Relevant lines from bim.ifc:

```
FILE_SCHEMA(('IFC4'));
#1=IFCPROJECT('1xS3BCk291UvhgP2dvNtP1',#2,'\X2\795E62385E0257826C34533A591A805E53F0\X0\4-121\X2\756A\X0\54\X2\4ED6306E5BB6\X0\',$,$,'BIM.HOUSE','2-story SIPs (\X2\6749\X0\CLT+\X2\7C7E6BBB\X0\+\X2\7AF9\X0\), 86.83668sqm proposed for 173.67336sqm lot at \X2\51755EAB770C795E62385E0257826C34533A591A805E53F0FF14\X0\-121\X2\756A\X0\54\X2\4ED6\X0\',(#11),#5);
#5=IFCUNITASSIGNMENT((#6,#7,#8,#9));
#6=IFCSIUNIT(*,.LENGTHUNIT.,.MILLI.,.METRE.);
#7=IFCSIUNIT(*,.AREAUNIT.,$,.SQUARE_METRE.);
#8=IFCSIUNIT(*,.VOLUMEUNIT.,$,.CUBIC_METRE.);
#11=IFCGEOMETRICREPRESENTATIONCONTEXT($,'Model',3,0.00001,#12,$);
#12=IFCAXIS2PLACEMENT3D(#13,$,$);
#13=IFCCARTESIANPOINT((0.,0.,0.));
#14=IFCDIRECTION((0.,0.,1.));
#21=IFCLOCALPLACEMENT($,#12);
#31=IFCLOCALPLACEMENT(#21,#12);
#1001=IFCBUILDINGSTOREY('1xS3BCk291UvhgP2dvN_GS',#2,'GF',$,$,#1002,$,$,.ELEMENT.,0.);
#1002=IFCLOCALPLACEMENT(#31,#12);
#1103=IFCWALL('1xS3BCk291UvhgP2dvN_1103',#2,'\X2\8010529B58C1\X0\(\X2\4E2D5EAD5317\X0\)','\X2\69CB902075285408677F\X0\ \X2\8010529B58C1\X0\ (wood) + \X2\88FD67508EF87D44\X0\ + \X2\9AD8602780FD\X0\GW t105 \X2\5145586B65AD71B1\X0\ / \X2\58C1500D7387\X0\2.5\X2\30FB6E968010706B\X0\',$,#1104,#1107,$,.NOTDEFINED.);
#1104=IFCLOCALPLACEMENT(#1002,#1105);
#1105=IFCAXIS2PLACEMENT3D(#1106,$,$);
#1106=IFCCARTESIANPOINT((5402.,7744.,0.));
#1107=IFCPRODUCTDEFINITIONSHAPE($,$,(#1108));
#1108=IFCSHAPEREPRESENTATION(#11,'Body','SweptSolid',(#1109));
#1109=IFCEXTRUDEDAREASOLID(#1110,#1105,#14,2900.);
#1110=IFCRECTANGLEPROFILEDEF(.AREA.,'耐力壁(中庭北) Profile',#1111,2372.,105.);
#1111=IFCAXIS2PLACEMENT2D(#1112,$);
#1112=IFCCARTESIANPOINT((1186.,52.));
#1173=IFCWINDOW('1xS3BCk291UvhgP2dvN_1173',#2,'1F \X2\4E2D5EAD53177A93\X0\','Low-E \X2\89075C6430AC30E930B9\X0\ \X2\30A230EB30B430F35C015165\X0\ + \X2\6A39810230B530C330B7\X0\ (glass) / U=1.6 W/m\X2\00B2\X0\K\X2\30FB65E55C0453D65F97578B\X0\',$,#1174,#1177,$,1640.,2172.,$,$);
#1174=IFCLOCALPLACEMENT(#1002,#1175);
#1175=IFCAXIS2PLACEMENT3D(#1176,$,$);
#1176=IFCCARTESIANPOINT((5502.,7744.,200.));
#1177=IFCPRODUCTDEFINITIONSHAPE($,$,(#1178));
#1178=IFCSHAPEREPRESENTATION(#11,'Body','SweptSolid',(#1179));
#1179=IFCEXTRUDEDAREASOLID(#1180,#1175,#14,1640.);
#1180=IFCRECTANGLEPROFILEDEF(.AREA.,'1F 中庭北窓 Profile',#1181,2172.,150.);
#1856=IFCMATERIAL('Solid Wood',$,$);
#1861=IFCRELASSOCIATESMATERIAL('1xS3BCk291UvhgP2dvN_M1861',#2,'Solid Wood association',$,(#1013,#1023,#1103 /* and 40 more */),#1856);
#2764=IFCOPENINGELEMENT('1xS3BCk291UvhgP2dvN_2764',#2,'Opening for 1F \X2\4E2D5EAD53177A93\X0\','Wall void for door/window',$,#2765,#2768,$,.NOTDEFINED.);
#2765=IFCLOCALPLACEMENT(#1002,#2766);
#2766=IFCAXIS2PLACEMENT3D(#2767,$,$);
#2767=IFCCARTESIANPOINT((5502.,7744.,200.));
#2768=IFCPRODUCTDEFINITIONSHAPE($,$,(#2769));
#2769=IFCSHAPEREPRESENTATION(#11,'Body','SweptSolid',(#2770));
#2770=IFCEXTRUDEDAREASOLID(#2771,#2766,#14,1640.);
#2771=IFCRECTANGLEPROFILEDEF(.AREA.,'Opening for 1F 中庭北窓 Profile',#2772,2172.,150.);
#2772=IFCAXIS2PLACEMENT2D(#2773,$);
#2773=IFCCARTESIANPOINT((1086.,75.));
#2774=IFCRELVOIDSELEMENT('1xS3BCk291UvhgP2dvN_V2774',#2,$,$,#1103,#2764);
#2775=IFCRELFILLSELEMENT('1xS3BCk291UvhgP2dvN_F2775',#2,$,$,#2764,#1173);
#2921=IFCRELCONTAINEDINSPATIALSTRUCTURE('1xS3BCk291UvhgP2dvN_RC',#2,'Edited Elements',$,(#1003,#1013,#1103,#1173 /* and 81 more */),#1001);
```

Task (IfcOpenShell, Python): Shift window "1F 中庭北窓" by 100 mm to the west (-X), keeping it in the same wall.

```python
import ifcopenshell
import ifcopenshell.api.geometry
import ifcopenshell.util.placement

model = ifcopenshell.open("bim.ifc")

window = model.by_guid("1xS3BCk291UvhgP2dvN_1173")
opening = window.FillsVoids[0].RelatingOpeningElement
wall = opening.VoidsElements[0].RelatingBuildingElement

wall_matrix = ifcopenshell.util.placement.get_local_placement(wall.ObjectPlacement)
shift = wall_matrix[:3, 0] * -100.0
before = ifcopenshell.util.placement.get_local_placement(window.ObjectPlacement)[:3, 3].copy()

# The window is not placed relative to its opening, so move both.
for product in (opening, window):
    matrix = ifcopenshell.util.placement.get_local_placement(product.ObjectPlacement)
    matrix[:3, 3] += shift
    ifcopenshell.api.geometry.edit_object_placement(model, product=product, matrix=matrix, is_si=False)

after = ifcopenshell.util.placement.get_local_placement(window.ObjectPlacement)[:3, 3]
print("window moved by", (after - before).round(3) + 0.0)

model.write("bim-out.ifc")
```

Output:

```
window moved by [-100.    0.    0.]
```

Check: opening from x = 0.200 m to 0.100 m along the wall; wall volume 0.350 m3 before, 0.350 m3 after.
